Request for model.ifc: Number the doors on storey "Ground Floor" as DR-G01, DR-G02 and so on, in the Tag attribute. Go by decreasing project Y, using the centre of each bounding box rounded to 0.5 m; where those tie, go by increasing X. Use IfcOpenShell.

First a look at what the model holds.

```python
import ifcopenshell
import ifcopenshell.util.element
import ifcopenshell.util.placement

model = ifcopenshell.open("model.ifc")
print(model.schema)
storey = next(s for s in model.by_type("IfcBuildingStorey") if s.Name == "Ground Floor")
doors = [e for e in ifcopenshell.util.element.get_decomposition(storey) if e.is_a("IfcDoor")]
for e in sorted(doors, key=lambda e: e.id()):
    origin = ifcopenshell.util.placement.get_local_placement(e.ObjectPlacement)[:3, 3]
    print(e.id(), e.Tag, e.Name, origin.round(2) + 0.0, sep=" | ")
```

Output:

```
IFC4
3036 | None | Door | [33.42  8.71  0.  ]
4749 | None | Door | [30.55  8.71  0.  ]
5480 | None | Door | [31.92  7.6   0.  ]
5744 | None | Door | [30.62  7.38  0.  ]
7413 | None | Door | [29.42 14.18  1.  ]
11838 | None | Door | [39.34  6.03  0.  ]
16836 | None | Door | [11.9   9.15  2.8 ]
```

```python
import ifcopenshell
import ifcopenshell.geom
import ifcopenshell.util.element
import ifcopenshell.util.shape

model = ifcopenshell.open("model.ifc")
settings = ifcopenshell.geom.settings()
settings.set("use-world-coords", True)


def centre(element):
    shape = ifcopenshell.geom.create_shape(settings, element)
    return ifcopenshell.util.shape.get_bbox_centroid(shape.geometry)


storey = next(s for s in model.by_type("IfcBuildingStorey") if s.Name == "Ground Floor")
doors = [e for e in ifcopenshell.util.element.get_decomposition(storey) if e.is_a("IfcDoor")]

# Insertion points can sit at a corner or the storey origin, so sort by the geometry (in metres).
centres = {e: centre(e) for e in doors}
doors.sort(key=lambda e: (-round(centres[e][1] / 0.5), centres[e][0]))

for i, e in enumerate(doors, start=1):
    number = f"DR-G{i:02d}"
    e.Tag = number
    print(e.id(), number)

model.write("model_rev.ifc")
```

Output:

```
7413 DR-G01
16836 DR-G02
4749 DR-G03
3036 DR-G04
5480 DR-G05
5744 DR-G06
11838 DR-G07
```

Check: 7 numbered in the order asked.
